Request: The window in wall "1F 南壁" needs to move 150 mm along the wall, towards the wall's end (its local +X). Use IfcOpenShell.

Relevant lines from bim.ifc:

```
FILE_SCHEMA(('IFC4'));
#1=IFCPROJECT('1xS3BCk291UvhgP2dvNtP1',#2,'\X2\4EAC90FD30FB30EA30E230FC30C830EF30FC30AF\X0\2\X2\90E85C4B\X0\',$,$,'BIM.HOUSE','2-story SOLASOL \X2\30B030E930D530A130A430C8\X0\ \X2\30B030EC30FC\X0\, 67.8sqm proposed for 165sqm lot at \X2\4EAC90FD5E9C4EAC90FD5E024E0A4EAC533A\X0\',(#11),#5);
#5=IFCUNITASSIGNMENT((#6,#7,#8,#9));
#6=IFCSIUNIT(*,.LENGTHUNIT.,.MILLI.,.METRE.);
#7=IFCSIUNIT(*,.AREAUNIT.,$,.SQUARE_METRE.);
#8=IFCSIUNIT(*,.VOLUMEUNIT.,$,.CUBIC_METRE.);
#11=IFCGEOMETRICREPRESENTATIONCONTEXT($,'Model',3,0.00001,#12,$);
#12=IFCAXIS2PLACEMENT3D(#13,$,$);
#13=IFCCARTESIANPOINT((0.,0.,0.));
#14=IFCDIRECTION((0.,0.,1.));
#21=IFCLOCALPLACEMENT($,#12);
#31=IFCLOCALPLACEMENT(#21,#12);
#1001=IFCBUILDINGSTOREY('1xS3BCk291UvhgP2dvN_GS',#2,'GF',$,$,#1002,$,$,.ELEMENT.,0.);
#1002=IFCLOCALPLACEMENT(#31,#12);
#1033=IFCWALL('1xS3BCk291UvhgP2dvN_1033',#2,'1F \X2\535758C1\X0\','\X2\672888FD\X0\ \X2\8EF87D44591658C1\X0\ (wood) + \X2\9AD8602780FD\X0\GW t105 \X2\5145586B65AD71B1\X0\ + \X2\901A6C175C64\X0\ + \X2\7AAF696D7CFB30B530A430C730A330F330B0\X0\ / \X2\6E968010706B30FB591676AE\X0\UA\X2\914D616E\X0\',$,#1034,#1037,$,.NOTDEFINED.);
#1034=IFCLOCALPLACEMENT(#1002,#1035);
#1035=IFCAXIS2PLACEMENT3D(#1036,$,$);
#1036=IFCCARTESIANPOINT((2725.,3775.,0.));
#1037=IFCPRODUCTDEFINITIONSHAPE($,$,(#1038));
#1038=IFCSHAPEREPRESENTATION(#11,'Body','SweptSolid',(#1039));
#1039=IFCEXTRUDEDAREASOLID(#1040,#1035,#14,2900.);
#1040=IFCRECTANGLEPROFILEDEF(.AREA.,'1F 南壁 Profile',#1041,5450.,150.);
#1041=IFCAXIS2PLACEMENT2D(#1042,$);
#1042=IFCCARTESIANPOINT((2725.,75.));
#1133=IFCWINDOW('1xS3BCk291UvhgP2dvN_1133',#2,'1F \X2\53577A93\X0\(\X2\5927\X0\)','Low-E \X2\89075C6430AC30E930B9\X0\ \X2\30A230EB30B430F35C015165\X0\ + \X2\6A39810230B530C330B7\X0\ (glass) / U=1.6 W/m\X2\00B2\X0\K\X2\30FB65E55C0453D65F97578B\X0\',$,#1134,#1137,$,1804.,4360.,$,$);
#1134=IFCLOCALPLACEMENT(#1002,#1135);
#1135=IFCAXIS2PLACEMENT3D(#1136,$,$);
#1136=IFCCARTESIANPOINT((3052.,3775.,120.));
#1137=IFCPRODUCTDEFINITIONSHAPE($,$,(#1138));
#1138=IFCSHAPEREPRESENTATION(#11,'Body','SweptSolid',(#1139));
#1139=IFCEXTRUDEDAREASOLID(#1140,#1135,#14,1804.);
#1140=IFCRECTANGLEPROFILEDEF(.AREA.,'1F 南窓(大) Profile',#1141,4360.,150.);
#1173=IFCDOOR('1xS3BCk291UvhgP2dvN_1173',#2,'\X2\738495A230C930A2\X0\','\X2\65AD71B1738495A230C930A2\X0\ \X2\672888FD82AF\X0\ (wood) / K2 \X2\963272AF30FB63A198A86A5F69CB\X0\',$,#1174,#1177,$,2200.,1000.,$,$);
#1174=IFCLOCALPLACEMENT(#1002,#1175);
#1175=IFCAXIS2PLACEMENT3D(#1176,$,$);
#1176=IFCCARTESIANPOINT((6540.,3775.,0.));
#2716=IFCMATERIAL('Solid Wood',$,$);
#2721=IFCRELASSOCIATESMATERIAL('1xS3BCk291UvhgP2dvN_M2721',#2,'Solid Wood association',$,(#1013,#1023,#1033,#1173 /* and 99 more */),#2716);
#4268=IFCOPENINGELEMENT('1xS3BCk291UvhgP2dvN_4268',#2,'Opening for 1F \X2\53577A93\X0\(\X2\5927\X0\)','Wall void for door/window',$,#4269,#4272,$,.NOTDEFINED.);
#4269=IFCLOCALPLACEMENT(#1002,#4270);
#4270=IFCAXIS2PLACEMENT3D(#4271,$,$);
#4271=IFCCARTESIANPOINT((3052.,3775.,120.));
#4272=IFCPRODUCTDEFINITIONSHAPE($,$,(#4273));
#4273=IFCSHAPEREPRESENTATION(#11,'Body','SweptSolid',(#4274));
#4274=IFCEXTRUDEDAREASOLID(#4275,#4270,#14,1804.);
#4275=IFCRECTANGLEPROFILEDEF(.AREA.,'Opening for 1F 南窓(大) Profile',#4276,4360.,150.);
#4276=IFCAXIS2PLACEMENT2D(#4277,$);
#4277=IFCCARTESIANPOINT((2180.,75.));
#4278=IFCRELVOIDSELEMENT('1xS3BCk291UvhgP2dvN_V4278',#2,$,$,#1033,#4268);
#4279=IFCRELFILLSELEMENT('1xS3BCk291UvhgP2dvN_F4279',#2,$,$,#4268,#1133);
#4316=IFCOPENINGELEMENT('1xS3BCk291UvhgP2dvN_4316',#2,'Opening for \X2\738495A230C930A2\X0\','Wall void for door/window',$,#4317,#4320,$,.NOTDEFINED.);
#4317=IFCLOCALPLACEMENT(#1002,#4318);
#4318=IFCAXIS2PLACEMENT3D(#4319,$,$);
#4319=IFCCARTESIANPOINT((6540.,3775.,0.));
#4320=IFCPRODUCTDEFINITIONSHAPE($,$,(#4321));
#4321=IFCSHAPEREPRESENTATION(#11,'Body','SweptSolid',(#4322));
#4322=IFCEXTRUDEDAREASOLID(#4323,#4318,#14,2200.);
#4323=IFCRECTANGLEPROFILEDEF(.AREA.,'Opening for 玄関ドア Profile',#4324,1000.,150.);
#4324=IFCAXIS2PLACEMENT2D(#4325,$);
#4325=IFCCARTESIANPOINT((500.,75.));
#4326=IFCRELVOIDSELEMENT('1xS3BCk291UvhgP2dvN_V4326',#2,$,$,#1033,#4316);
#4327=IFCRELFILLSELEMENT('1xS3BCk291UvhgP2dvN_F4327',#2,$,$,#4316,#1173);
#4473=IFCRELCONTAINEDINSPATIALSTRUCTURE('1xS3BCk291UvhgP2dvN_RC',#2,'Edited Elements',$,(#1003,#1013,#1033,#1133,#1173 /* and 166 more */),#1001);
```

```python
import ifcopenshell
import ifcopenshell.api.geometry
import ifcopenshell.util.placement
import ifcopenshell.util.unit

model = ifcopenshell.open("bim.ifc")
unit_scale = ifcopenshell.util.unit.calculate_unit_scale(model)

window = model.by_guid("1xS3BCk291UvhgP2dvN_1133")
opening = window.FillsVoids[0].RelatingOpeningElement
wall = opening.VoidsElements[0].RelatingBuildingElement

wall_matrix = ifcopenshell.util.placement.get_local_placement(wall.ObjectPlacement)
shift = wall_matrix[:3, 0] * 0.15 / unit_scale
before = ifcopenshell.util.placement.get_local_placement(window.ObjectPlacement)[:3, 3].copy()

# The window is not placed relative to its opening, so move both.
for product in (opening, window):
    matrix = ifcopenshell.util.placement.get_local_placement(product.ObjectPlacement)
    matrix[:3, 3] += shift
    ifcopenshell.api.geometry.edit_object_placement(model, product=product, matrix=matrix, is_si=False)

after = ifcopenshell.util.placement.get_local_placement(window.ObjectPlacement)[:3, 3]
print("window moved by", (after - before).round(3) + 0.0)

model.write("bim_updated.ifc")
```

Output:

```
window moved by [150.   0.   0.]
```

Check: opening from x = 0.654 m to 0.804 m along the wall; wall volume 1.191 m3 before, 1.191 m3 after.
